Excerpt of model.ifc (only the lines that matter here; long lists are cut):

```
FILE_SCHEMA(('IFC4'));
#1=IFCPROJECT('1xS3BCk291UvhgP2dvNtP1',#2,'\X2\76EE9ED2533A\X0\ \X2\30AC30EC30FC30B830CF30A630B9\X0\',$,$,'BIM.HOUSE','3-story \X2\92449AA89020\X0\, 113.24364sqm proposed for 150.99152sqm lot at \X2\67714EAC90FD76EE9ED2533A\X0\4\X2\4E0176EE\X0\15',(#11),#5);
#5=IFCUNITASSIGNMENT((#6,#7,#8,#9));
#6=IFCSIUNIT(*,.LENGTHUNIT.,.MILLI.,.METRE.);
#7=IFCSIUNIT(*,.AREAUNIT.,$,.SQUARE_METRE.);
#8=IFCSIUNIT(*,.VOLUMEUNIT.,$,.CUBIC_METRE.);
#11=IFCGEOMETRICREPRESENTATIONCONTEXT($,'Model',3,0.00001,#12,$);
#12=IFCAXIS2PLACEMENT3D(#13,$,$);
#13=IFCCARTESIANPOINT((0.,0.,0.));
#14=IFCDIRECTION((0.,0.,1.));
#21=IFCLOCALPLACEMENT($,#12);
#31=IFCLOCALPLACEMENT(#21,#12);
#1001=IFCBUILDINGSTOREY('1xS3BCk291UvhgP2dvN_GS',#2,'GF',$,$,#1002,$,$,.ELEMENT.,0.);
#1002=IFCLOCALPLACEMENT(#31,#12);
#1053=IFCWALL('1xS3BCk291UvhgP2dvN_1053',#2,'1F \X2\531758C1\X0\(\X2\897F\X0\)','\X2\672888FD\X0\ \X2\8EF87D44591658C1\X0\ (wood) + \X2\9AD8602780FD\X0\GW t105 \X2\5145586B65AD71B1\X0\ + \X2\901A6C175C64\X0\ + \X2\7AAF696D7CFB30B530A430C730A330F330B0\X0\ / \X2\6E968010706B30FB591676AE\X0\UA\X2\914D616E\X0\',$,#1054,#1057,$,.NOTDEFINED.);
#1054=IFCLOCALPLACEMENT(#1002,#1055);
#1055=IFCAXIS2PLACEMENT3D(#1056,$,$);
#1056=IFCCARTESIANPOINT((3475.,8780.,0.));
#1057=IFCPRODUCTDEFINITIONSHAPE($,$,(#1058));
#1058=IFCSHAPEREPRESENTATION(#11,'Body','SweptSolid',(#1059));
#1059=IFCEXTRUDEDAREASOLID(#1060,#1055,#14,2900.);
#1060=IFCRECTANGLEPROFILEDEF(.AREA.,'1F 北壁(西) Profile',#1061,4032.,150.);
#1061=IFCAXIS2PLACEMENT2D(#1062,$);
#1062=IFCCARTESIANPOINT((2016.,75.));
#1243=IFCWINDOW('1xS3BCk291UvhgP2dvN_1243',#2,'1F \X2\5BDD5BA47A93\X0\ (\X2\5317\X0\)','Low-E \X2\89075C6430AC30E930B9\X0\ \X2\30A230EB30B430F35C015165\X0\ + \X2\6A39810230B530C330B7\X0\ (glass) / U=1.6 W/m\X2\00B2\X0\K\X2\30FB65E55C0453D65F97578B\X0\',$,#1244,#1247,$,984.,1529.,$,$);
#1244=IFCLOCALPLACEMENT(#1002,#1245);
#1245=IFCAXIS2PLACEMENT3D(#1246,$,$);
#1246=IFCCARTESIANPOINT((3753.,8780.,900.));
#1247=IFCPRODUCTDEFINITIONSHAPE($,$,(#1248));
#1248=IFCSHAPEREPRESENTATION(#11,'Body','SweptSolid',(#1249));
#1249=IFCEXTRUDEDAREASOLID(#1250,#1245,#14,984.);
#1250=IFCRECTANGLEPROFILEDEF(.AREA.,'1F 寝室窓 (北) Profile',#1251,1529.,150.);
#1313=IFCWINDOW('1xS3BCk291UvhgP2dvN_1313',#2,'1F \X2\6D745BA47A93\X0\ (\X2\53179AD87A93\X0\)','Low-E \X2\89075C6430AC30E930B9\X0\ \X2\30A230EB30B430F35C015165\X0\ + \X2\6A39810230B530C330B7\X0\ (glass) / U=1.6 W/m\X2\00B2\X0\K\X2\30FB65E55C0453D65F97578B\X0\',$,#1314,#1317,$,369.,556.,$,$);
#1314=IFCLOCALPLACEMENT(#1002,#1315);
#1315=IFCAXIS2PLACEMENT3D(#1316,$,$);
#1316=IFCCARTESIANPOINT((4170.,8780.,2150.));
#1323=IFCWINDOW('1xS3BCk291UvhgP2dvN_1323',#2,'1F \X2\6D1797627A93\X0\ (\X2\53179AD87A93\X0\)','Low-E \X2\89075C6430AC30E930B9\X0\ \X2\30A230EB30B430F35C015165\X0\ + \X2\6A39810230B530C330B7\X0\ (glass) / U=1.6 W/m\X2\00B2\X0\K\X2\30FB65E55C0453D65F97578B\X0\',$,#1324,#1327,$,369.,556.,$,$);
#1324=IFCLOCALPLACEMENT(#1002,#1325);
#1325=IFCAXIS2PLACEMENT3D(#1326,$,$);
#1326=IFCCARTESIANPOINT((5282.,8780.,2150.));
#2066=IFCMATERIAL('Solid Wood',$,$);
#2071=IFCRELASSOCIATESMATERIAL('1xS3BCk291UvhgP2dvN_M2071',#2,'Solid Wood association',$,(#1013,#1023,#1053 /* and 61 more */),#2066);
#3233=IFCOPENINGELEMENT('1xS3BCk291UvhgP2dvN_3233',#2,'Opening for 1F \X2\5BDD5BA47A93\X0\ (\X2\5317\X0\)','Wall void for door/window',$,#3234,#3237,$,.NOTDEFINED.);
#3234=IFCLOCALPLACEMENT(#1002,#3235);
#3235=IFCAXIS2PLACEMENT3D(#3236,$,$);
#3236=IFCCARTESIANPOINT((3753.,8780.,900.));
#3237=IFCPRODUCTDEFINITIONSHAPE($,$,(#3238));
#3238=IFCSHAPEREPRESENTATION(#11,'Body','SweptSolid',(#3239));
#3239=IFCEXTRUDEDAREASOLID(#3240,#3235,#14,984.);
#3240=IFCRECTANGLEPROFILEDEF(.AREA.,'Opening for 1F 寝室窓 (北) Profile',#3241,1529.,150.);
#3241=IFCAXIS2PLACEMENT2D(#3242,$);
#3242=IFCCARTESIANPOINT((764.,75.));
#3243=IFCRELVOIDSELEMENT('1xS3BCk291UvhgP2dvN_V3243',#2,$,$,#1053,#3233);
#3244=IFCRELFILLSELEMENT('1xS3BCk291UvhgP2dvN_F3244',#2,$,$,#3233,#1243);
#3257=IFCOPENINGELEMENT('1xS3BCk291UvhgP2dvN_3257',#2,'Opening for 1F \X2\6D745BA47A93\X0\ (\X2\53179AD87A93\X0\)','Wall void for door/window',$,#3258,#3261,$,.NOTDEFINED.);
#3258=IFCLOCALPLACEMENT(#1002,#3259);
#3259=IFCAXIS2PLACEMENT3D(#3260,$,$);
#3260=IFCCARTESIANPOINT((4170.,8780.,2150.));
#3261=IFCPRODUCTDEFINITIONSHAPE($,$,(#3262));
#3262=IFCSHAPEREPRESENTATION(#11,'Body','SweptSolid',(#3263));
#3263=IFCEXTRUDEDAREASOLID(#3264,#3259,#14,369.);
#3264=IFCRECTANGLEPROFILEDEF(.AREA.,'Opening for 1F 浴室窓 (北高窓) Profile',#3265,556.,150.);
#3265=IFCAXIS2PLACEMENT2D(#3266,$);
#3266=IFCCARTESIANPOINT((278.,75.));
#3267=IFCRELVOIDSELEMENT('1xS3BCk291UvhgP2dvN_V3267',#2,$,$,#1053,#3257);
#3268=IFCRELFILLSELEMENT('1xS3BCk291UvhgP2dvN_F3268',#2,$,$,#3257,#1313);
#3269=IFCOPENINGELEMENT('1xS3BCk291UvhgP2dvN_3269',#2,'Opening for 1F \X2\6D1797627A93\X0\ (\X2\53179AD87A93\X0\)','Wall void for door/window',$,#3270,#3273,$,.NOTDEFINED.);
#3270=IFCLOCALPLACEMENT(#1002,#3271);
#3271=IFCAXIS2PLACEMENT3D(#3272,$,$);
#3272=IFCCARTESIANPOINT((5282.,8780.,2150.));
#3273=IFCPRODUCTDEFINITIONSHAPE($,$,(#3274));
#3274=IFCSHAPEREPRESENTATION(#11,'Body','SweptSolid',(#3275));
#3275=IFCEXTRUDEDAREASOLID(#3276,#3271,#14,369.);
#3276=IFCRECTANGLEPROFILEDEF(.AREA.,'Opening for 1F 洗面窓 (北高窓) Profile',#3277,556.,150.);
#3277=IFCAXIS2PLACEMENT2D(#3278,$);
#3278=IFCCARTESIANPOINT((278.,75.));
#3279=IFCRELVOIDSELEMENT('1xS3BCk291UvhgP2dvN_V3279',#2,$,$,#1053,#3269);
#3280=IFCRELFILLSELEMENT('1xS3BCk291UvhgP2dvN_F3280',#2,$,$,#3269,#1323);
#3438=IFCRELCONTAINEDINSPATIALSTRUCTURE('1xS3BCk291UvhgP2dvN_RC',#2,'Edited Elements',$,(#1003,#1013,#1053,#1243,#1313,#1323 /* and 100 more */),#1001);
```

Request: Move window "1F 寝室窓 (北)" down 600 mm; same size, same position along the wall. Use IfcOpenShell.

```python
import numpy as np
import ifcopenshell
import ifcopenshell.api.geometry
import ifcopenshell.util.placement
import ifcopenshell.util.unit

model = ifcopenshell.open("model.ifc")
unit_scale = ifcopenshell.util.unit.calculate_unit_scale(model)

window = model.by_guid("1xS3BCk291UvhgP2dvN_1243")
opening = window.FillsVoids[0].RelatingOpeningElement
dz = -600.0

shift = np.array([0.0, 0.0, dz])
# The window is not placed relative to its opening, so move both.
for product in (opening, window):
    matrix = ifcopenshell.util.placement.get_local_placement(product.ObjectPlacement)
    matrix[:3, 3] += shift
    ifcopenshell.api.geometry.edit_object_placement(model, product=product, matrix=matrix, is_si=False)

print(f"moved by {dz * unit_scale:+.3f} m")

model.write("model_updated.ifc")
```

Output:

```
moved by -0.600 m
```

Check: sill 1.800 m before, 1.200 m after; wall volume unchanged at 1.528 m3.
